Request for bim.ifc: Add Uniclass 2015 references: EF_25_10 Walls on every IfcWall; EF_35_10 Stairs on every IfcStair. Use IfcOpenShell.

First a look at what the model holds.

```python
import ifcopenshell

model = ifcopenshell.open("bim.ifc")
print(model.schema)
print("classifications:", [c.Name for c in model.by_type("IfcClassification")])
for ifc_class in ("IfcDoor", "IfcRoof", "IfcStair", "IfcWall", "IfcWindow"):
    print(ifc_class, len(model.by_type(ifc_class)))
```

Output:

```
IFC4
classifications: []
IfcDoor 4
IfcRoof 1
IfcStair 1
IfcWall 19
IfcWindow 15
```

```python
import ifcopenshell
import ifcopenshell.api.classification

model = ifcopenshell.open("bim.ifc")

system = ifcopenshell.api.classification.add_classification(model, classification="Uniclass 2015")

codes = {
    "IfcWall": ("EF_25_10", "Walls"),
    "IfcStair": ("EF_35_10", "Stairs"),
}
for ifc_class, (code, name) in codes.items():
    products = model.by_type(ifc_class)
    ifcopenshell.api.classification.add_reference(
        model, products=products, classification=system, identification=code, name=name
    )
    print(code, len(products))

model.write("bim_edited.ifc")
```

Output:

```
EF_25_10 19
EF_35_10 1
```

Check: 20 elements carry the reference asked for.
